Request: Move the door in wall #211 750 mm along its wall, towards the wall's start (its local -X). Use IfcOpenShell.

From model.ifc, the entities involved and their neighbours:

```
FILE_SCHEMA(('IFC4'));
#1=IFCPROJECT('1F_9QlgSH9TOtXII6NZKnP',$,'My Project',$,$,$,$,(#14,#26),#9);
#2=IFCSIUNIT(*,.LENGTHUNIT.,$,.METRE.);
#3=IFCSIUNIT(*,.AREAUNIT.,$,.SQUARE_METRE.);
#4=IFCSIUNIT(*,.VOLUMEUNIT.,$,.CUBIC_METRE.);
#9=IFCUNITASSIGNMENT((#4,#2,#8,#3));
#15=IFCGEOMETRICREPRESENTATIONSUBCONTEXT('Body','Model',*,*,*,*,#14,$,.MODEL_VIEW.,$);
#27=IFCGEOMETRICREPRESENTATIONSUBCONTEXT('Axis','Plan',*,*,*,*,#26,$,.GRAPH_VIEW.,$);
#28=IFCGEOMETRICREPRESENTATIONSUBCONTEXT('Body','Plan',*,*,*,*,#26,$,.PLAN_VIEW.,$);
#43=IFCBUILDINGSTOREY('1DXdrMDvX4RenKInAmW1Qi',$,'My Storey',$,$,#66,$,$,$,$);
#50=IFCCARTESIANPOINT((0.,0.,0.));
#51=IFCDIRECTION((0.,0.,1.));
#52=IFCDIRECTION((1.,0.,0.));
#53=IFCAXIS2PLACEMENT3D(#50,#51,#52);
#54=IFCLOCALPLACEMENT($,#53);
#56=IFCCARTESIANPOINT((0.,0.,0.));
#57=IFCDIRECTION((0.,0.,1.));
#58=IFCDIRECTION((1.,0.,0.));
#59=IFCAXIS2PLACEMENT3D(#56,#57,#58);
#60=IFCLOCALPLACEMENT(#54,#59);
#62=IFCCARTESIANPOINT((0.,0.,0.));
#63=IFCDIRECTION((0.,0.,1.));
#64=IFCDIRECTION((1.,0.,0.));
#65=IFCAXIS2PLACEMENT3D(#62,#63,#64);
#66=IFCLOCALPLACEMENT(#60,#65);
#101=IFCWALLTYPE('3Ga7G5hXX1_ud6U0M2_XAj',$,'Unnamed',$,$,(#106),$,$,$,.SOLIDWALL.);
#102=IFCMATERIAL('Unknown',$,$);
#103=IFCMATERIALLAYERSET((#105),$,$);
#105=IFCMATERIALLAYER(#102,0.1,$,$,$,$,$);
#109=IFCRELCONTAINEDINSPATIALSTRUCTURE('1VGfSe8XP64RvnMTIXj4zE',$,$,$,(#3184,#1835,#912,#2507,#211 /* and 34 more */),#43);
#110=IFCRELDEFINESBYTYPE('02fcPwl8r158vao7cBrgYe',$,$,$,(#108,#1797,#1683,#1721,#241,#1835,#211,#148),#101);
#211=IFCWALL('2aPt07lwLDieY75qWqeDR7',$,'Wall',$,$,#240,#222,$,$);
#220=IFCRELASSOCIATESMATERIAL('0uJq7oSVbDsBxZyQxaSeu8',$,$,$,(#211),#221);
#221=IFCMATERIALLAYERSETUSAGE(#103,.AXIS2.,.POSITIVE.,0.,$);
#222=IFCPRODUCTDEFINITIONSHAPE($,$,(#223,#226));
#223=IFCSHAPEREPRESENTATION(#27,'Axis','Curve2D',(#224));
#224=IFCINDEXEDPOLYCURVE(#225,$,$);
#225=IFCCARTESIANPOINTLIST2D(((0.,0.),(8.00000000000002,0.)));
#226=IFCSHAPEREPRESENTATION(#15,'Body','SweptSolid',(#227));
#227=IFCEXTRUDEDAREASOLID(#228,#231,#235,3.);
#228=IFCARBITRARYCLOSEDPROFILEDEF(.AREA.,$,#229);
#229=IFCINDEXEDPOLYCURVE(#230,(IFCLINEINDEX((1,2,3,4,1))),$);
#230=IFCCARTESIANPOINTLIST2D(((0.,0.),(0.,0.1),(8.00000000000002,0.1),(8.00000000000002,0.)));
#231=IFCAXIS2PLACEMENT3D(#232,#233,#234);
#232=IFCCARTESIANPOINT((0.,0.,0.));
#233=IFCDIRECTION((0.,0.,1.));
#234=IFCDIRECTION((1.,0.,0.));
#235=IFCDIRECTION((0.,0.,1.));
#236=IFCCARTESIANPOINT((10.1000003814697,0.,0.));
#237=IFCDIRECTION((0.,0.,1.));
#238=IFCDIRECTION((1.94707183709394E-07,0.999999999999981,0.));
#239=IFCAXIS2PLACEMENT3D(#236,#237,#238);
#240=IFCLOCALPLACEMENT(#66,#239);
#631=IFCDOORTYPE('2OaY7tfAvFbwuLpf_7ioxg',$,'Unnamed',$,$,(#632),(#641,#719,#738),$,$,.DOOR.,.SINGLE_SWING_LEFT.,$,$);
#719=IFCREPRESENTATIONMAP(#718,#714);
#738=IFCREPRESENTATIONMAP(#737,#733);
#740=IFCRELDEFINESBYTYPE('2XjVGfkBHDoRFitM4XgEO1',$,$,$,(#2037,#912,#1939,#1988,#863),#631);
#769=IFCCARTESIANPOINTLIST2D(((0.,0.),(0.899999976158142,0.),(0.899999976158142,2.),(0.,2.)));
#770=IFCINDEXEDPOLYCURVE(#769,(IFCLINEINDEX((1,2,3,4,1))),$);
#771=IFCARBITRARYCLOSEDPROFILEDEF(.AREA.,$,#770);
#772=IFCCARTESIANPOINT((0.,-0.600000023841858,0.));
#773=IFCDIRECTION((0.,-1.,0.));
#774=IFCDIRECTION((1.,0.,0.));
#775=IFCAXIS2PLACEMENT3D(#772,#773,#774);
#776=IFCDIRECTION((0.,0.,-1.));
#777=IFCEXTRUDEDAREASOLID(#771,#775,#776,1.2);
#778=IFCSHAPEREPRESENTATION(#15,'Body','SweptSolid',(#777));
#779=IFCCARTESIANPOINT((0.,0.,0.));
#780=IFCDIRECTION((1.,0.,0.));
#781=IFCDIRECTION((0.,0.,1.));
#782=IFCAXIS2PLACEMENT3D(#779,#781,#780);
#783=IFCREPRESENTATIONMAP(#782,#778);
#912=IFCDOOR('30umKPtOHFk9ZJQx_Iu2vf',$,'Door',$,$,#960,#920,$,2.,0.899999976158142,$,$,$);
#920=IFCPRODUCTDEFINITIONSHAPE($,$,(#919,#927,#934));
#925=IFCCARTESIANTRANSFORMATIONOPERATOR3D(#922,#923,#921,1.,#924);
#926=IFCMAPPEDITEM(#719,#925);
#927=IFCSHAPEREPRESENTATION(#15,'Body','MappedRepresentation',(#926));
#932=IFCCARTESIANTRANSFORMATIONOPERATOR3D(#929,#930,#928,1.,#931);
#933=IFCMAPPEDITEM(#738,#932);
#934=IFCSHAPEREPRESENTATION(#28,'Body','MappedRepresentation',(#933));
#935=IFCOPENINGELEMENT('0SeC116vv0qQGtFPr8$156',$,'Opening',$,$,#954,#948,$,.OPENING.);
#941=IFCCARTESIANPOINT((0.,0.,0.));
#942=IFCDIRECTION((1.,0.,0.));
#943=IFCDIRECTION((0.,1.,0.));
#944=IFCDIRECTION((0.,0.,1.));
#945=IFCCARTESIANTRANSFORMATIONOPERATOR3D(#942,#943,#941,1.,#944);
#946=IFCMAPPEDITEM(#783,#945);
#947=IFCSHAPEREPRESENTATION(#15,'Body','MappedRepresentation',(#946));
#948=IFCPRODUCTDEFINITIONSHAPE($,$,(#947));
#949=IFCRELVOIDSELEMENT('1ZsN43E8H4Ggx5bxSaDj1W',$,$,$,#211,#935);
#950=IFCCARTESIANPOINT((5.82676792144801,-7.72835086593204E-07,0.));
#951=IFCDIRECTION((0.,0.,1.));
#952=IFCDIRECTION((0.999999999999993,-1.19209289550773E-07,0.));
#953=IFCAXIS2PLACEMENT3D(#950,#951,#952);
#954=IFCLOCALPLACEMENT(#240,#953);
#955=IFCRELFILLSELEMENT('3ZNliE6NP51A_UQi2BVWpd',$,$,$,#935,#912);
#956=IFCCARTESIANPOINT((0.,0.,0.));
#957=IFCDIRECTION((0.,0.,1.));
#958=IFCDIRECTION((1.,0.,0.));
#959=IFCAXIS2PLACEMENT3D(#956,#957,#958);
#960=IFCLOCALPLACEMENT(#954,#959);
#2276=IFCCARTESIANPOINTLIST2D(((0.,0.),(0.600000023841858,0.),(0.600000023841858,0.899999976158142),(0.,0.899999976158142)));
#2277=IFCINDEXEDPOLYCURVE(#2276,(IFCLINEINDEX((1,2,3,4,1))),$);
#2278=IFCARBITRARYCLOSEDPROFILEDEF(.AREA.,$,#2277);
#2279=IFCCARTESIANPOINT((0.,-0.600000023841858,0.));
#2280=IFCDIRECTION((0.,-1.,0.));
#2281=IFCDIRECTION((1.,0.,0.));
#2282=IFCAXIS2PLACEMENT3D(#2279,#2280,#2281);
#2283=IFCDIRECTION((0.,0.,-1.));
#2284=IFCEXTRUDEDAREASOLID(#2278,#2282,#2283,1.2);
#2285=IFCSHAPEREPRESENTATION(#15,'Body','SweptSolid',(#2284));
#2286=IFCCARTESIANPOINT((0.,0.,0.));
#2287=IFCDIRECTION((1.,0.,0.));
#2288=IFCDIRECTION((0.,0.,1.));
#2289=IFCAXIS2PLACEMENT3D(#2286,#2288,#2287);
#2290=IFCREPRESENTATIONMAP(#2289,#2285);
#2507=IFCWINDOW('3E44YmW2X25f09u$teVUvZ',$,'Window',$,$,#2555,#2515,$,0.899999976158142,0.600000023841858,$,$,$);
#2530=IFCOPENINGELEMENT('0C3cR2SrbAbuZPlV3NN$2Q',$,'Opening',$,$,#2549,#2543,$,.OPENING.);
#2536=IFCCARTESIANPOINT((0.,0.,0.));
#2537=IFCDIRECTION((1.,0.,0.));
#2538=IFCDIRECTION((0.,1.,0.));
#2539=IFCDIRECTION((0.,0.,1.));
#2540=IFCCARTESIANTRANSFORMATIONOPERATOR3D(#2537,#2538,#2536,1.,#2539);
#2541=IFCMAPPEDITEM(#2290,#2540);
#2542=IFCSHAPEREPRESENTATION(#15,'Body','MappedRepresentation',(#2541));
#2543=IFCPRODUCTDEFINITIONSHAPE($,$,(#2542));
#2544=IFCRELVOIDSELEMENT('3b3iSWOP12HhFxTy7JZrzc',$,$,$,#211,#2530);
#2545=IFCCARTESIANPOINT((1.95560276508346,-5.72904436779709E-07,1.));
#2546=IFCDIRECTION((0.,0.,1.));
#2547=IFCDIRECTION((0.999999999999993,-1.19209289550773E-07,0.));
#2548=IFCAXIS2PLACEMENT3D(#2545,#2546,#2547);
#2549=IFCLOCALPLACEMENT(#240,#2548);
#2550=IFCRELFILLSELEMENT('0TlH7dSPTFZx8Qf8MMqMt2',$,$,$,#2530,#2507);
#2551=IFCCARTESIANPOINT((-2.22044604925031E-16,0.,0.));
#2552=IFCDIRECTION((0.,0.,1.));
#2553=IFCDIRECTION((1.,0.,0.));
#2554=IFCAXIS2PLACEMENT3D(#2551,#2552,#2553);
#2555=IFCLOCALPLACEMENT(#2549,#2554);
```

```python
import ifcopenshell
import ifcopenshell.api.geometry
import ifcopenshell.util.placement
import ifcopenshell.util.unit

model = ifcopenshell.open("model.ifc")
unit_scale = ifcopenshell.util.unit.calculate_unit_scale(model)

door = model.by_guid("30umKPtOHFk9ZJQx_Iu2vf")
opening = door.FillsVoids[0].RelatingOpeningElement
wall = opening.VoidsElements[0].RelatingBuildingElement

wall_matrix = ifcopenshell.util.placement.get_local_placement(wall.ObjectPlacement)
shift = wall_matrix[:3, 0] * -0.75 / unit_scale
before = ifcopenshell.util.placement.get_local_placement(door.ObjectPlacement)[:3, 3].copy()

# The door is placed relative to its opening, so it follows when the opening moves.
matrix = ifcopenshell.util.placement.get_local_placement(opening.ObjectPlacement)
matrix[:3, 3] += shift
ifcopenshell.api.geometry.edit_object_placement(
    model, product=opening, matrix=matrix, is_si=False, should_transform_children=True
)

after = ifcopenshell.util.placement.get_local_placement(door.ObjectPlacement)[:3, 3]
print("door moved by", (after - before).round(3) + 0.0)

model.write("model-out.ifc")
```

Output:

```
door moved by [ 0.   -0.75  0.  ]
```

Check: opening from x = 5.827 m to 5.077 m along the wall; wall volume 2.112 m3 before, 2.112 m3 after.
